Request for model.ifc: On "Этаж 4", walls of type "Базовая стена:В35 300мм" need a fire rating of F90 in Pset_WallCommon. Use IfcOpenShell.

First a look at what the model holds.

```python
import ifcopenshell
import ifcopenshell.util.element

model = ifcopenshell.open("model.ifc")
print(model.schema)
storey = next(s for s in model.by_type("IfcBuildingStorey") if s.Name == "Этаж 4")
walls = [e for e in ifcopenshell.util.element.get_decomposition(storey) if e.is_a("IfcWall")]
seen = {}
for e in walls:
    element_type = ifcopenshell.util.element.get_type(e)
    key = (element_type.Name if element_type != e and element_type else None, ifcopenshell.util.element.get_pset(e, "Pset_WallCommon", "FireRating"))
    seen[key] = seen.get(key, 0) + 1
for (name, value), count in sorted(seen.items(), key=str):
    print(count, "x", name, "|", value)
```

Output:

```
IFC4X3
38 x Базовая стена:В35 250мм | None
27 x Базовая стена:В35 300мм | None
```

```python
import ifcopenshell
import ifcopenshell.api.pset
import ifcopenshell.util.element

model = ifcopenshell.open("model.ifc")

storey = next(s for s in model.by_type("IfcBuildingStorey") if s.Name == "Этаж 4")
walls = [e for e in ifcopenshell.util.element.get_decomposition(storey) if e.is_a("IfcWall")]

count = 0
for e in walls:
    element_type = ifcopenshell.util.element.get_type(e)
    if element_type in (None, e) or element_type.Name != "Базовая стена:В35 300мм":
        continue
    # add_pset returns the element's existing set when there is one.
    pset = ifcopenshell.api.pset.add_pset(model, product=e, name="Pset_WallCommon")
    ifcopenshell.api.pset.edit_pset(model, pset=pset, properties={"FireRating": "F90"})
    count += 1

print(count, "walls updated")

model.write("model_v2.ifc")
```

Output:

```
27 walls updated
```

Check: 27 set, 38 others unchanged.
